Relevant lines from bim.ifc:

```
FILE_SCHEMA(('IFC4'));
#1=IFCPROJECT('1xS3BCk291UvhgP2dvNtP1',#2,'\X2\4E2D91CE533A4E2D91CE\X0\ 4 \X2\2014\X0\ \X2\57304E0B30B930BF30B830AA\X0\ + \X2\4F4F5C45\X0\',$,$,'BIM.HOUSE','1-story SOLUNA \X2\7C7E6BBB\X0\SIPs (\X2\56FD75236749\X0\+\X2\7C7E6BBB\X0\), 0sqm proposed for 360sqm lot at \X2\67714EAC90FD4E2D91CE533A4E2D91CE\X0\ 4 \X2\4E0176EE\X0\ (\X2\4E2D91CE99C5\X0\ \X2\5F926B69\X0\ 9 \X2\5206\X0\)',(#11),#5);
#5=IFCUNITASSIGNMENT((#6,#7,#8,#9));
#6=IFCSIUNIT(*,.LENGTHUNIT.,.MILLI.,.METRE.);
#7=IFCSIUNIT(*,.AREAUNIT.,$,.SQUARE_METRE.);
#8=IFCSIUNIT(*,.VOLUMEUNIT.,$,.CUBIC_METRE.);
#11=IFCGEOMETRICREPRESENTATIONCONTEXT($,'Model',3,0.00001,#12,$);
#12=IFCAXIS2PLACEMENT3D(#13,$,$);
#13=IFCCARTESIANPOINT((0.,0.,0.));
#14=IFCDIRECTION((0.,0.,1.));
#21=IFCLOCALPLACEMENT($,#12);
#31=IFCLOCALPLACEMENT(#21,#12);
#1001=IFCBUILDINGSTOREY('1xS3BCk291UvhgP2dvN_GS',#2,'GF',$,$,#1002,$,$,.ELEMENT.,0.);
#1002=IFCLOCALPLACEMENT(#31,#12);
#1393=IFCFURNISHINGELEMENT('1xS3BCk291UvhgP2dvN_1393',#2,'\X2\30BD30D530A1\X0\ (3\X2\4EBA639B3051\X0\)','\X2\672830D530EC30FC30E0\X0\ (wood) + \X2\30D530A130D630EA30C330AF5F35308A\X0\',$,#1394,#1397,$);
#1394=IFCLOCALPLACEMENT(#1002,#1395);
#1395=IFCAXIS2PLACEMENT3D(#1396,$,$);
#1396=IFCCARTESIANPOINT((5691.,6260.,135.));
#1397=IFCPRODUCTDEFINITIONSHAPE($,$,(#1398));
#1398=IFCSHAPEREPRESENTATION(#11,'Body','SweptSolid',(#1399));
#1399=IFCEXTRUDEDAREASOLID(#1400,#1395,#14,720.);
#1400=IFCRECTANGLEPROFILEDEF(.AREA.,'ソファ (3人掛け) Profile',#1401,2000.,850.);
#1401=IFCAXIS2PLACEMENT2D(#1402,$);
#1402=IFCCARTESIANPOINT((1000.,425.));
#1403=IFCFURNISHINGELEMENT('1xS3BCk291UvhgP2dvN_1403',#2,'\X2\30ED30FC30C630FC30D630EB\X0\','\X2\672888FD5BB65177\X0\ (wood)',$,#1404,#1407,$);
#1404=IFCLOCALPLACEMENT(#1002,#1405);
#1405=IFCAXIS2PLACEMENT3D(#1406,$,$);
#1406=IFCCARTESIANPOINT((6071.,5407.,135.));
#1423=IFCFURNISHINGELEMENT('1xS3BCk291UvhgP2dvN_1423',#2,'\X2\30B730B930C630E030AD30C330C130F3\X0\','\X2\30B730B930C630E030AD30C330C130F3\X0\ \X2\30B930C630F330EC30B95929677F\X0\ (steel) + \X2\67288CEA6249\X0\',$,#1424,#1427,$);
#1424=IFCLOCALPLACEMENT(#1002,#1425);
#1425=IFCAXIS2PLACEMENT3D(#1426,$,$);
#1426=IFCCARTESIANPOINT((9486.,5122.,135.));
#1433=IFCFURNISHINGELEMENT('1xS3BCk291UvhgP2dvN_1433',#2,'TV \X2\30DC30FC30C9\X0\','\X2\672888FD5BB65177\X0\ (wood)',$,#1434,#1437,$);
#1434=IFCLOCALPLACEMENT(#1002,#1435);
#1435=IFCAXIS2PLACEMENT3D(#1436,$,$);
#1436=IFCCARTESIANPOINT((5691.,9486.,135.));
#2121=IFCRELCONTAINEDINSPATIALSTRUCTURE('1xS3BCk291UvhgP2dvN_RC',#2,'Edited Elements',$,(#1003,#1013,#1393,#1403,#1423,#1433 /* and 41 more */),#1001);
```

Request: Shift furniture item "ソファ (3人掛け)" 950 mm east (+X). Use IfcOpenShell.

```python
import ifcopenshell
import ifcopenshell.api.geometry
import ifcopenshell.util.placement

model = ifcopenshell.open("bim.ifc")

item = model.by_guid("1xS3BCk291UvhgP2dvN_1393")
matrix = ifcopenshell.util.placement.get_local_placement(item.ObjectPlacement)
matrix[0, 3] += 950.0
ifcopenshell.api.geometry.edit_object_placement(model, product=item, matrix=matrix, is_si=False)

print(ifcopenshell.util.placement.get_local_placement(item.ObjectPlacement).round(3) + 0.0)

model.write("bim_updated.ifc")
```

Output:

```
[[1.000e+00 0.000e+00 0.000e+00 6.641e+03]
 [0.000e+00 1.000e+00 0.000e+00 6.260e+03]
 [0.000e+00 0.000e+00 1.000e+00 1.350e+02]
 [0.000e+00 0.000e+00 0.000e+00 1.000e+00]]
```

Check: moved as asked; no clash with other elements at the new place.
